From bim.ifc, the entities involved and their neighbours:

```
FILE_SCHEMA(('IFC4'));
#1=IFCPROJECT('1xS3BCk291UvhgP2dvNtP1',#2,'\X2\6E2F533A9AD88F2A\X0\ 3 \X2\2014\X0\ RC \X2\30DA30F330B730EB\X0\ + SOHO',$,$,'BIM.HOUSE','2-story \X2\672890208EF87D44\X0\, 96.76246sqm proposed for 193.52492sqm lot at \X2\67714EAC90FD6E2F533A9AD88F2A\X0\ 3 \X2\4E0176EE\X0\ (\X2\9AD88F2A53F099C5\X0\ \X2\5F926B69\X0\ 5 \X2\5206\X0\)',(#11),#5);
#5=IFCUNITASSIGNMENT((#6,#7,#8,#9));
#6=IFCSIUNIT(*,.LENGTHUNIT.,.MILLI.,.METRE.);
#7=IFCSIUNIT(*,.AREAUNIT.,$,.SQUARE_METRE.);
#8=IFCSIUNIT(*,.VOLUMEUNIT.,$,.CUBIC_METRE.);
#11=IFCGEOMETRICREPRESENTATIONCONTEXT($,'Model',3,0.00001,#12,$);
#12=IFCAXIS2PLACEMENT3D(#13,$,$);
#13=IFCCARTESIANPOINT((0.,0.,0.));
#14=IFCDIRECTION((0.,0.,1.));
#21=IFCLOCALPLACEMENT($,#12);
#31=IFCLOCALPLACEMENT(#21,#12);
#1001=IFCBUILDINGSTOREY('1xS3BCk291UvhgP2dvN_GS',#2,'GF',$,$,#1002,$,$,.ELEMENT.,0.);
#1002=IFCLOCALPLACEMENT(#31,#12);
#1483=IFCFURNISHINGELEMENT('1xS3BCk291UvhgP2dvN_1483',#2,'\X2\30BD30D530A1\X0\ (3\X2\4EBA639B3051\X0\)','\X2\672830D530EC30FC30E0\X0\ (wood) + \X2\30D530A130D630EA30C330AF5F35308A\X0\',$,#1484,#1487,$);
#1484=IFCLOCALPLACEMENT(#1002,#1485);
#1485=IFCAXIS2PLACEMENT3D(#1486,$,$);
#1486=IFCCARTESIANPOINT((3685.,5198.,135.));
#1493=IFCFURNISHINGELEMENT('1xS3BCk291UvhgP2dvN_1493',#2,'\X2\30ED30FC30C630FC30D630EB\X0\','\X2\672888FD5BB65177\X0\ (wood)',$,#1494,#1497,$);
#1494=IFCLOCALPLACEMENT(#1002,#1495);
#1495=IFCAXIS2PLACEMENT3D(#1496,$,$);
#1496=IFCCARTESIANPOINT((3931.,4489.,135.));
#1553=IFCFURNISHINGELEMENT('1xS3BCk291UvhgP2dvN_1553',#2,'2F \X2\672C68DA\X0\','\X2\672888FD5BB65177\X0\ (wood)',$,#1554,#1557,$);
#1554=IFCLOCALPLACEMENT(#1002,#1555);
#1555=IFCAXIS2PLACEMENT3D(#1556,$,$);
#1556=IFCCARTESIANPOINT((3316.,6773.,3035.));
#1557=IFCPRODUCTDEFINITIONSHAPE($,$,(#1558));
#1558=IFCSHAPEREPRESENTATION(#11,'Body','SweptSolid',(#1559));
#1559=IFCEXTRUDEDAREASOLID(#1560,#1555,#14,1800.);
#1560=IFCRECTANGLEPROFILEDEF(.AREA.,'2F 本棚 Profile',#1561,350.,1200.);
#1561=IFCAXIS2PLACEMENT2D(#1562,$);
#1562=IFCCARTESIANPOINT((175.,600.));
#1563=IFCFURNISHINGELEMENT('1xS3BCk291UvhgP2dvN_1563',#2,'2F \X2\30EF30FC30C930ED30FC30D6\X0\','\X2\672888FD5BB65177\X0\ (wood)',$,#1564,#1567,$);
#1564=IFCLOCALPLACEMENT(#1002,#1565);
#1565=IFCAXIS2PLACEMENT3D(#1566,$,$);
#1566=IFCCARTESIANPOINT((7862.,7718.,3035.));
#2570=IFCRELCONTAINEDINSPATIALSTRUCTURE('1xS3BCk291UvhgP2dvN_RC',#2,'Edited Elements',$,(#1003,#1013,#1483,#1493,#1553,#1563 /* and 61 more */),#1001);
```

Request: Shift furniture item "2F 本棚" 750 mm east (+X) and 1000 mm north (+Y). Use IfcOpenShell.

```python
import ifcopenshell
import ifcopenshell.api.geometry
import ifcopenshell.util.placement
import ifcopenshell.util.unit

model = ifcopenshell.open("bim.ifc")
unit_scale = ifcopenshell.util.unit.calculate_unit_scale(model)

item = model.by_guid("1xS3BCk291UvhgP2dvN_1553")
matrix = ifcopenshell.util.placement.get_local_placement(item.ObjectPlacement)
matrix[0, 3] += 0.75 / unit_scale
matrix[1, 3] += 1 / unit_scale
ifcopenshell.api.geometry.edit_object_placement(model, product=item, matrix=matrix, is_si=False)

print(ifcopenshell.util.placement.get_local_placement(item.ObjectPlacement).round(3) + 0.0)

model.write("bim_v2.ifc")
```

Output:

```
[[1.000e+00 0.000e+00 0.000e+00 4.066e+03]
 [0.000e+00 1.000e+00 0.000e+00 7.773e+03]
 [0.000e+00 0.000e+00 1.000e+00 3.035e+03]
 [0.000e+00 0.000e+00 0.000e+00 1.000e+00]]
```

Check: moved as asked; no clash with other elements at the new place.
